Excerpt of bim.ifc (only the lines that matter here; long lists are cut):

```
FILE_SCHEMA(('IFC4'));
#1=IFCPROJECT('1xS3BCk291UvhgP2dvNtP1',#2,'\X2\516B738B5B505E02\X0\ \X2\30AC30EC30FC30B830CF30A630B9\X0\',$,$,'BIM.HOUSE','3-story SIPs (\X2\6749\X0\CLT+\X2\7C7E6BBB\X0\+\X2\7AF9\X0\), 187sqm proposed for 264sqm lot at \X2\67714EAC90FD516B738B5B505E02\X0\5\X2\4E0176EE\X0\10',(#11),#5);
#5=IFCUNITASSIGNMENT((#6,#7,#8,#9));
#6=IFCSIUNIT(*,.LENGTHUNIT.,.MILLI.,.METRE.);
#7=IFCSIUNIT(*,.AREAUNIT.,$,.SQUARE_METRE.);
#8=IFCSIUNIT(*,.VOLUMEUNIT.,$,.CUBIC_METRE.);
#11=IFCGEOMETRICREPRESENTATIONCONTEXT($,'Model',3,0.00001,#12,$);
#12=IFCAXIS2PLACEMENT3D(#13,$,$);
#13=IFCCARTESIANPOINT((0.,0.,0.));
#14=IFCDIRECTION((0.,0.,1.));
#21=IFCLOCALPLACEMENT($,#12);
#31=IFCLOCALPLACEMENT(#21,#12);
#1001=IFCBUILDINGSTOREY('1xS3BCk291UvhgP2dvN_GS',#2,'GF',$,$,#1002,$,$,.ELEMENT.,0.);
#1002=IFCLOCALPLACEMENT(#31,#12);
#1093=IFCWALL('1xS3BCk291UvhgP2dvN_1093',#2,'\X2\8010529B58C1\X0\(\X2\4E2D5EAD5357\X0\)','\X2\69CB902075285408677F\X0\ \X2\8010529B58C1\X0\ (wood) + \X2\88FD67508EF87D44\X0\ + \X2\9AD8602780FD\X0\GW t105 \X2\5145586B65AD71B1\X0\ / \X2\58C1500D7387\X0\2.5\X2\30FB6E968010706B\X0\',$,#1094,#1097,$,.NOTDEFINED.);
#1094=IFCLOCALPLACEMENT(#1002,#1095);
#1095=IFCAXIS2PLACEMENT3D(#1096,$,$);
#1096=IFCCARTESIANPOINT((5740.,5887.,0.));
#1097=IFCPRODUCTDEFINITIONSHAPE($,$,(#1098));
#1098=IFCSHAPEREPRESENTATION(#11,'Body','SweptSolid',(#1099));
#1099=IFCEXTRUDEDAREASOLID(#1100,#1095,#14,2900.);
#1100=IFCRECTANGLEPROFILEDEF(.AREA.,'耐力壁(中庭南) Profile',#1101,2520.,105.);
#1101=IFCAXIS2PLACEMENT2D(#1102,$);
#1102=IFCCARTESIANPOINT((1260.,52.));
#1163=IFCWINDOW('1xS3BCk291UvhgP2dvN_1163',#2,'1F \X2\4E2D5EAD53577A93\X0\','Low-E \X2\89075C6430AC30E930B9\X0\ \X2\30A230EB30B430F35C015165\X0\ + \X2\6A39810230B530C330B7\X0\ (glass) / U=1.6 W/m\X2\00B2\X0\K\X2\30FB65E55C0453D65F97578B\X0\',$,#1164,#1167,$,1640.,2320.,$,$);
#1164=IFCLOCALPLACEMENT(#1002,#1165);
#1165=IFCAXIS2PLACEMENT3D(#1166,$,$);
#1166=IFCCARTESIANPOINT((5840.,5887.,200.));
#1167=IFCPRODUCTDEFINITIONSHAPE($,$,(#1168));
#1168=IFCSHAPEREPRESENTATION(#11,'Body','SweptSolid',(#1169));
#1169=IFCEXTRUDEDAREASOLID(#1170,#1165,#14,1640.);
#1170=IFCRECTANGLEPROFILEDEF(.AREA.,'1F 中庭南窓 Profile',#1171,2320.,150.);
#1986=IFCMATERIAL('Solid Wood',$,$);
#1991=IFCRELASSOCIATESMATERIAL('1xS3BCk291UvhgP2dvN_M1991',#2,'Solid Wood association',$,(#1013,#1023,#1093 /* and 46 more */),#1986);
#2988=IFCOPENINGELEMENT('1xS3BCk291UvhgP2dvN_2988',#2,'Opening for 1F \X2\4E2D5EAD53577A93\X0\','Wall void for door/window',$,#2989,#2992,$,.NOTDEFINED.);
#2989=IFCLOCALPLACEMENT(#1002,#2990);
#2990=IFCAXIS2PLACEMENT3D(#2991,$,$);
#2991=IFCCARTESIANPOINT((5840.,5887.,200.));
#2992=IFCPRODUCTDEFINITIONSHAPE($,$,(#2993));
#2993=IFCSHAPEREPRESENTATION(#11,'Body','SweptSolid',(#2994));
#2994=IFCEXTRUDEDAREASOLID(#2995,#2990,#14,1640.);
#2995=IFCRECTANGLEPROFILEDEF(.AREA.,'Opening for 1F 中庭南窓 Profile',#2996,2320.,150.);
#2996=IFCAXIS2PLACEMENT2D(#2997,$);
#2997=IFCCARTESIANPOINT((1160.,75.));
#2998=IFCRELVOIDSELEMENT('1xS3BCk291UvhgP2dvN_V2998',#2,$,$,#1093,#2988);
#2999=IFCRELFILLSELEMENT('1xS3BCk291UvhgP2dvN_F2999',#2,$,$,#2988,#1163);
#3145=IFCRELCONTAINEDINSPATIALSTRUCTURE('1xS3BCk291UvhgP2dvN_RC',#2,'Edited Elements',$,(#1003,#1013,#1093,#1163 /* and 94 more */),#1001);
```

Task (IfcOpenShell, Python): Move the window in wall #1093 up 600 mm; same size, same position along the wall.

```python
import numpy as np
import ifcopenshell
import ifcopenshell.api.geometry
import ifcopenshell.util.placement
import ifcopenshell.util.unit

model = ifcopenshell.open("bim.ifc")
unit_scale = ifcopenshell.util.unit.calculate_unit_scale(model)

window = model.by_guid("1xS3BCk291UvhgP2dvN_1163")
opening = window.FillsVoids[0].RelatingOpeningElement
dz = 0.6 / unit_scale

shift = np.array([0.0, 0.0, dz])
# The window is not placed relative to its opening, so move both.
for product in (opening, window):
    matrix = ifcopenshell.util.placement.get_local_placement(product.ObjectPlacement)
    matrix[:3, 3] += shift
    ifcopenshell.api.geometry.edit_object_placement(model, product=product, matrix=matrix, is_si=False)

print(f"moved by {dz * unit_scale:+.3f} m")

model.write("bim_updated.ifc")
```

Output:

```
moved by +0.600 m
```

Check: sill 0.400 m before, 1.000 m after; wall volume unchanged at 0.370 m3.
